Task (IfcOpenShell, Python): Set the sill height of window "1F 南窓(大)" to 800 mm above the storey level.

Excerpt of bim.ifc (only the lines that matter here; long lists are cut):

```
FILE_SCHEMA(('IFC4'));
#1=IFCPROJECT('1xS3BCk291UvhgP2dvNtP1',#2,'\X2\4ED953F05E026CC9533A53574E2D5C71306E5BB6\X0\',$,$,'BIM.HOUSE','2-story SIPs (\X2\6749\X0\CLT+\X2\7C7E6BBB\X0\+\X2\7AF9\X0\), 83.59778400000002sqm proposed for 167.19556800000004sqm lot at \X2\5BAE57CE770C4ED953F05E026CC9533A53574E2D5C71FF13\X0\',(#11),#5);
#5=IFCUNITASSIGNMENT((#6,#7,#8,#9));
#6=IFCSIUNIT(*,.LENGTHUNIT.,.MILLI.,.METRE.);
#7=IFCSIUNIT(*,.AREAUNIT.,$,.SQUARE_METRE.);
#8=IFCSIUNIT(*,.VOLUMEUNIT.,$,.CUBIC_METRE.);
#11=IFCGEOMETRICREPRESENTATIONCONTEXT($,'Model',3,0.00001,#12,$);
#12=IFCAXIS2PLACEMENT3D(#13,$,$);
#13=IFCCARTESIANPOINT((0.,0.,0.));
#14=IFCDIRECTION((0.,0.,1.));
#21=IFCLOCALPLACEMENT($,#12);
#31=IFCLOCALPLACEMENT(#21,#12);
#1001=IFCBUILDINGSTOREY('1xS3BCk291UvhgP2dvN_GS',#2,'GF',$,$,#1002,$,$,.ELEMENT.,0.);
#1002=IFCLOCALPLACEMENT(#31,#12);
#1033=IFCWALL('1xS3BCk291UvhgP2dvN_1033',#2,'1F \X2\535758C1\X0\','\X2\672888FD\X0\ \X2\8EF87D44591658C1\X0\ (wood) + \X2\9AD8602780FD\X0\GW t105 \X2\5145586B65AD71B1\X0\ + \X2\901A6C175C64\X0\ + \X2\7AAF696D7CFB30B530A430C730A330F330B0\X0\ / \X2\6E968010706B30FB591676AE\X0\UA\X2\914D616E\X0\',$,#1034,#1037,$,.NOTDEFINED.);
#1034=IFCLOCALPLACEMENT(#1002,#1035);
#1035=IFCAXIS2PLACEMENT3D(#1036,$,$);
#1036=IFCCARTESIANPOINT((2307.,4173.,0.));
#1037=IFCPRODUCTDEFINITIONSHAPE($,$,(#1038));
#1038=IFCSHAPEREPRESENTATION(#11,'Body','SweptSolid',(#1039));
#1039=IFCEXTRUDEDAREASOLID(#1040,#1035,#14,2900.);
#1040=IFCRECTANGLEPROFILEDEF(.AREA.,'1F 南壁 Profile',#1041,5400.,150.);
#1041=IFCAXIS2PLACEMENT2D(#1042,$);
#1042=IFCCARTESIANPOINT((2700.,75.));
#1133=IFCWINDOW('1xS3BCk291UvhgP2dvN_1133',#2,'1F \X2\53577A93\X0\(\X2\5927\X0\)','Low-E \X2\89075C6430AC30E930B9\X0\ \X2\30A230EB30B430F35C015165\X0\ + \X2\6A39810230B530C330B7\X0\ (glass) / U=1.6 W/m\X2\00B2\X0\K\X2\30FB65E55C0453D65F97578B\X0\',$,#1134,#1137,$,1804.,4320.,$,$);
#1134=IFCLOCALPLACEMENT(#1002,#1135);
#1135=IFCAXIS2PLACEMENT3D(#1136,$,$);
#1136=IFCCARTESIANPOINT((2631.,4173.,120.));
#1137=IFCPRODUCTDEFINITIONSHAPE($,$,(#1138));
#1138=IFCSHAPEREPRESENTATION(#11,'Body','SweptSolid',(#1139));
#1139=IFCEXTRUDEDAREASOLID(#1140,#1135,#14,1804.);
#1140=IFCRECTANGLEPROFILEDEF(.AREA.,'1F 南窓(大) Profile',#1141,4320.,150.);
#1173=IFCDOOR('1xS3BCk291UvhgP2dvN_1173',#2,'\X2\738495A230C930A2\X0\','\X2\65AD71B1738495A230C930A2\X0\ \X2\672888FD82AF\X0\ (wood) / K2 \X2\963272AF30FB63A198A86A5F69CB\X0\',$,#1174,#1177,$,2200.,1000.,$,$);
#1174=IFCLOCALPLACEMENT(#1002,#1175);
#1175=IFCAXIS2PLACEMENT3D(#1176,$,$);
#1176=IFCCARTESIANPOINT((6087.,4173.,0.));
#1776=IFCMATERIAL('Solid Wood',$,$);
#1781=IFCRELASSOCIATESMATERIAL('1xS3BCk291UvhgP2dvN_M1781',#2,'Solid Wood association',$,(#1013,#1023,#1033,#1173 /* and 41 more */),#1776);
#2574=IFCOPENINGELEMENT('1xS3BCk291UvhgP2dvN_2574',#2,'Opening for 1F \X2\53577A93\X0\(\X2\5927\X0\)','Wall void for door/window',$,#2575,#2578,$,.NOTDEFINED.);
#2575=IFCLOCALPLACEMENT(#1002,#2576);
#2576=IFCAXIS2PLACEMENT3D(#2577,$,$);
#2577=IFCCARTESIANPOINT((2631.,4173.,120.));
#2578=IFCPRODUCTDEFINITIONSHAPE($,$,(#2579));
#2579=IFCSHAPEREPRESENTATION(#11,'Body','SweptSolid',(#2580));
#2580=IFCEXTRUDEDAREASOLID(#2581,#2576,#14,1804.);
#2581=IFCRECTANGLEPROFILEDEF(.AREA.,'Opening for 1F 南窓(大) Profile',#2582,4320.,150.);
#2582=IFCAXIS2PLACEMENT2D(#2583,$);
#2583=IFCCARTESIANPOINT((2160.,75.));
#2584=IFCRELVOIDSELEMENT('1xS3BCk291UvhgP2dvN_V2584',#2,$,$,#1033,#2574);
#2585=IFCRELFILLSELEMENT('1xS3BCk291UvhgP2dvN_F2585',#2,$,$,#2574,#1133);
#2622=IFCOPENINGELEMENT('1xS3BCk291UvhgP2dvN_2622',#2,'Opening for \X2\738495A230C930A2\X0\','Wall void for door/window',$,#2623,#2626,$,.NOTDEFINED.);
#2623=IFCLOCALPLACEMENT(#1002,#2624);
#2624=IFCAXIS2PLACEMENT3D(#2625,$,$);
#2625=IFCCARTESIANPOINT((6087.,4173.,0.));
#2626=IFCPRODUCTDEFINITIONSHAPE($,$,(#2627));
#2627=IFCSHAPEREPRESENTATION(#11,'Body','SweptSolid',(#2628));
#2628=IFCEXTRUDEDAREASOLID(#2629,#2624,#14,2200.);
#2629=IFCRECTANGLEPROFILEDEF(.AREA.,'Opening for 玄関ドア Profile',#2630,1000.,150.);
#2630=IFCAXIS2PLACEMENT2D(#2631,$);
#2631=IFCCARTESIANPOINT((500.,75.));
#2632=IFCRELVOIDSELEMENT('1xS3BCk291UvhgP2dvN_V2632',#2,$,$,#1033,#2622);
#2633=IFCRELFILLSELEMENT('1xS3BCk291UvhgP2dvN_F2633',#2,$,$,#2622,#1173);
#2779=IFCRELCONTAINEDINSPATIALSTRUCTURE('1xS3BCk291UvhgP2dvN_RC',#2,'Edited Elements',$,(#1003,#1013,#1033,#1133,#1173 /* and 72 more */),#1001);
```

```python
import numpy as np
import ifcopenshell
import ifcopenshell.api.geometry
import ifcopenshell.geom
import ifcopenshell.util.element
import ifcopenshell.util.placement
import ifcopenshell.util.shape
import ifcopenshell.util.unit

model = ifcopenshell.open("bim.ifc")
unit_scale = ifcopenshell.util.unit.calculate_unit_scale(model)

window = model.by_guid("1xS3BCk291UvhgP2dvN_1133")
opening = window.FillsVoids[0].RelatingOpeningElement
storey = ifcopenshell.util.element.get_container(window, ifc_class="IfcBuildingStorey")
level = ifcopenshell.util.placement.get_local_placement(storey.ObjectPlacement)[2, 3]

# The opening's origin need not be at the sill, so measure its lowest point.
shape = ifcopenshell.geom.create_shape(ifcopenshell.geom.settings(), opening)
bottom = ifcopenshell.util.shape.get_shape_bottom_elevation(shape, shape.geometry) / unit_scale
dz = level + 800.0 - bottom

shift = np.array([0.0, 0.0, dz])
# The window is not placed relative to its opening, so move both.
for product in (opening, window):
    matrix = ifcopenshell.util.placement.get_local_placement(product.ObjectPlacement)
    matrix[:3, 3] += shift
    ifcopenshell.api.geometry.edit_object_placement(model, product=product, matrix=matrix, is_si=False)

print(f"moved by {dz * unit_scale:+.3f} m")

model.write("bim_edited.ifc")
```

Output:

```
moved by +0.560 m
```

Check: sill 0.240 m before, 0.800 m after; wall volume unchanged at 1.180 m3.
